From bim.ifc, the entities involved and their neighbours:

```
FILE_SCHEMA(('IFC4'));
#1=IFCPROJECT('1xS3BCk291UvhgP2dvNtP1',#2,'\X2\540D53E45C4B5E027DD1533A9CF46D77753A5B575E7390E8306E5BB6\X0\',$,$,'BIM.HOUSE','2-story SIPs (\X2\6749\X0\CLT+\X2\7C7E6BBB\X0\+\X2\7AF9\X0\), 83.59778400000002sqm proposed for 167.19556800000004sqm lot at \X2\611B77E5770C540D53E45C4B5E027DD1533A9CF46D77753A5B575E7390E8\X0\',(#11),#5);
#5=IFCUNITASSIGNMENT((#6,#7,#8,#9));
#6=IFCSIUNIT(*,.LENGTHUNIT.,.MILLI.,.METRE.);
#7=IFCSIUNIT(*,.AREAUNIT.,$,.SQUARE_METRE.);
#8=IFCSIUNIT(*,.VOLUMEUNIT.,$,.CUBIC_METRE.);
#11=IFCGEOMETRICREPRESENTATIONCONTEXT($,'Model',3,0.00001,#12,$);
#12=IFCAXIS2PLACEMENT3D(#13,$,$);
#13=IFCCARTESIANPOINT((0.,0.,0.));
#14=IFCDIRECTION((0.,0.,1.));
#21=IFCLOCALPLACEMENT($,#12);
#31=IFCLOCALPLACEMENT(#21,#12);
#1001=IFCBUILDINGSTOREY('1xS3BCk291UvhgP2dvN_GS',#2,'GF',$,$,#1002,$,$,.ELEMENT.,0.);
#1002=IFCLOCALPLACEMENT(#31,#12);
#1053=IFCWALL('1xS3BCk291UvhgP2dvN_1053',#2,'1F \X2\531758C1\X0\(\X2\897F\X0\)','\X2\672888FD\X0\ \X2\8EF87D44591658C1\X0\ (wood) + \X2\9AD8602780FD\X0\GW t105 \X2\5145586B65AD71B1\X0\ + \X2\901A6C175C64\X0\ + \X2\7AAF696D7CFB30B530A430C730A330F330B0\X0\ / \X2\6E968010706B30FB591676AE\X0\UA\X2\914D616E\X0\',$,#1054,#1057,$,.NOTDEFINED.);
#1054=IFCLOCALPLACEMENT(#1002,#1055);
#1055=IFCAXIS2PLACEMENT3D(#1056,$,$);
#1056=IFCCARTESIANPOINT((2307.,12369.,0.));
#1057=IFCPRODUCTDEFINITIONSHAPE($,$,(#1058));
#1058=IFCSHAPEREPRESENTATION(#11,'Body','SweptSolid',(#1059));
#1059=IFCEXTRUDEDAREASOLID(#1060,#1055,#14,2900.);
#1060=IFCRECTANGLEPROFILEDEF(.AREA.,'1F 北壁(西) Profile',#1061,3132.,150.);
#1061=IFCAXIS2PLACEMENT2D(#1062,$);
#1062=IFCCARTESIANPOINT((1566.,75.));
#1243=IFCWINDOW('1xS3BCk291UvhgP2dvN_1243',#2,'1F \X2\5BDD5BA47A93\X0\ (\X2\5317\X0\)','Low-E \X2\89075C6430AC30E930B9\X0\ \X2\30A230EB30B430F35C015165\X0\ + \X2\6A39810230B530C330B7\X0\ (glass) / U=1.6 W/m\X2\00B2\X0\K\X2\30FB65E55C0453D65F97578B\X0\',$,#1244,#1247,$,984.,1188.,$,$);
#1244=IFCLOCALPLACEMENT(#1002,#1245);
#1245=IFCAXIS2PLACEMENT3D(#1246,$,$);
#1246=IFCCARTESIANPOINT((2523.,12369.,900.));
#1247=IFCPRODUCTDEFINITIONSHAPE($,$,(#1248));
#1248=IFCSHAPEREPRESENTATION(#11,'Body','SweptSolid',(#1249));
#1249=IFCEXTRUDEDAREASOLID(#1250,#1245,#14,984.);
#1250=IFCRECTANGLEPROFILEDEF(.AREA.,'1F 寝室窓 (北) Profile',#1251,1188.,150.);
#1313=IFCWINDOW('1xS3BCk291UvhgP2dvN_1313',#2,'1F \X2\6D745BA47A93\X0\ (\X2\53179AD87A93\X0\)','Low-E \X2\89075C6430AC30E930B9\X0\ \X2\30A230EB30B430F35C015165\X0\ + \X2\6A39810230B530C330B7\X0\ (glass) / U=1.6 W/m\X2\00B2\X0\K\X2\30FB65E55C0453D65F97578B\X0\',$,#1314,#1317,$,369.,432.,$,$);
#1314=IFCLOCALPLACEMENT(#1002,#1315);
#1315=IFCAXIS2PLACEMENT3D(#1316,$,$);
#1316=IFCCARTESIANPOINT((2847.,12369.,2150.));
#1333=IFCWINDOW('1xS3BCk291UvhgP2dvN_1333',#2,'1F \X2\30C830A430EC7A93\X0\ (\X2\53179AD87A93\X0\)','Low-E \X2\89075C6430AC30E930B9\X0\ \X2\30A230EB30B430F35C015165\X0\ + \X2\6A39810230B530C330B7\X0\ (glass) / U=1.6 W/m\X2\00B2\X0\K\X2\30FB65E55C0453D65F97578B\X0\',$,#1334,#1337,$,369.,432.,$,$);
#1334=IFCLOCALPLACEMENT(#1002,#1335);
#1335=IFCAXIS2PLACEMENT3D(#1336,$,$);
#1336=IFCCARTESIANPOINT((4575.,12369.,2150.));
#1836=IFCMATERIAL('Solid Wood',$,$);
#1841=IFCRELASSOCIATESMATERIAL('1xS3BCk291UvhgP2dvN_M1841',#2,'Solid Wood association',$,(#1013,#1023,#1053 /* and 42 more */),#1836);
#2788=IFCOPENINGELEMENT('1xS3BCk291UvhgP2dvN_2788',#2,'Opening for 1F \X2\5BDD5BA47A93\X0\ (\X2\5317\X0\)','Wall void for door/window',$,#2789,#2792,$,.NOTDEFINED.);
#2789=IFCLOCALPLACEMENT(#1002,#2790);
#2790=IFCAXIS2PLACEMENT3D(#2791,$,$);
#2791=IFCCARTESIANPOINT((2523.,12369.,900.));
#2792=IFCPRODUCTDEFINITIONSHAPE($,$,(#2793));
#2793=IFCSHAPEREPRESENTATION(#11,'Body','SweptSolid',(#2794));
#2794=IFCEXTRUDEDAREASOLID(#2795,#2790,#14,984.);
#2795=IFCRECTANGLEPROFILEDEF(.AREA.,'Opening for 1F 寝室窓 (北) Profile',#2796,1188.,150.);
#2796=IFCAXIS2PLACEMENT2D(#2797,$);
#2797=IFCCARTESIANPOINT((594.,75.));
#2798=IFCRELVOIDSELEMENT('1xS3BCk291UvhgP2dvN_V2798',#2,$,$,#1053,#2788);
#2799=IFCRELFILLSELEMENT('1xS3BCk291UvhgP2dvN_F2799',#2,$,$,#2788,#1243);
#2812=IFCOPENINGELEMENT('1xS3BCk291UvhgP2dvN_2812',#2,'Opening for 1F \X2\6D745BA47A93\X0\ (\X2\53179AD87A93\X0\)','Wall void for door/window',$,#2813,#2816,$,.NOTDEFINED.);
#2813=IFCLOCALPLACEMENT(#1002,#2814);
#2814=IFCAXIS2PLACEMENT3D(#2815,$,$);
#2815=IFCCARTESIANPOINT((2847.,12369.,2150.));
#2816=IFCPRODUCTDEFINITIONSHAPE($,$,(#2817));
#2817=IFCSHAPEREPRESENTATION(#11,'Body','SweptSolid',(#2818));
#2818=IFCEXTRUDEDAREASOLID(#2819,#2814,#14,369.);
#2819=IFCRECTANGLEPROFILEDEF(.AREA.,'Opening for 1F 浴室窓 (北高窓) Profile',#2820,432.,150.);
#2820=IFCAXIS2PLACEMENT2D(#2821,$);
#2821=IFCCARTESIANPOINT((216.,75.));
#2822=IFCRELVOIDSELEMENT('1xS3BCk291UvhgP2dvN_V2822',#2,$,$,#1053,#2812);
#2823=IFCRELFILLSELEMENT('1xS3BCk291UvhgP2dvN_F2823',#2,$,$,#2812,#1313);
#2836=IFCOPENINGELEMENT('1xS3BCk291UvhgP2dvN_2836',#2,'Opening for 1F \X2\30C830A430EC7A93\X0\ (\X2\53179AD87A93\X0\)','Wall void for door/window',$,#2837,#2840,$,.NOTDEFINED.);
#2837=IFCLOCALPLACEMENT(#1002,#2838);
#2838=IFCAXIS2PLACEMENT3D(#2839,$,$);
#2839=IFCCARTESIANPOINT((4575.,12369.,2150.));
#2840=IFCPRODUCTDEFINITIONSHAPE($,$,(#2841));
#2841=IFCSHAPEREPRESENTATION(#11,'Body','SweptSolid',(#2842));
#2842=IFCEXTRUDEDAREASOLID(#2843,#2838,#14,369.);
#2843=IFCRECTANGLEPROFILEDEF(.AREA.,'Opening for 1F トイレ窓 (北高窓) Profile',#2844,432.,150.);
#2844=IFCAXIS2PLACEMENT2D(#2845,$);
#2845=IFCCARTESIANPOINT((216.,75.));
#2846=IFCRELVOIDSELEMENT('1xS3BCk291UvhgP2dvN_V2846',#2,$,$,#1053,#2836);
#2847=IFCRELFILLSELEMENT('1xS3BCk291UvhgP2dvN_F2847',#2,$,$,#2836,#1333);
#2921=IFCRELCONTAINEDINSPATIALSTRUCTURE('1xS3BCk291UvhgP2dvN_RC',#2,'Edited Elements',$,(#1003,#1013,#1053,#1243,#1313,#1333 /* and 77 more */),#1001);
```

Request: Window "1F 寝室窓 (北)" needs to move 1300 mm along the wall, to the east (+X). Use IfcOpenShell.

```python
import ifcopenshell
import ifcopenshell.api.geometry
import ifcopenshell.util.placement
import ifcopenshell.util.unit

model = ifcopenshell.open("bim.ifc")
unit_scale = ifcopenshell.util.unit.calculate_unit_scale(model)

window = model.by_guid("1xS3BCk291UvhgP2dvN_1243")
opening = window.FillsVoids[0].RelatingOpeningElement
wall = opening.VoidsElements[0].RelatingBuildingElement

wall_matrix = ifcopenshell.util.placement.get_local_placement(wall.ObjectPlacement)
shift = wall_matrix[:3, 0] * 1.3 / unit_scale
before = ifcopenshell.util.placement.get_local_placement(window.ObjectPlacement)[:3, 3].copy()

# The window is not placed relative to its opening, so move both.
for product in (opening, window):
    matrix = ifcopenshell.util.placement.get_local_placement(product.ObjectPlacement)
    matrix[:3, 3] += shift
    ifcopenshell.api.geometry.edit_object_placement(model, product=product, matrix=matrix, is_si=False)

after = ifcopenshell.util.placement.get_local_placement(window.ObjectPlacement)[:3, 3]
print("window moved by", (after - before).round(3) + 0.0)

model.write("bim_v2.ifc")
```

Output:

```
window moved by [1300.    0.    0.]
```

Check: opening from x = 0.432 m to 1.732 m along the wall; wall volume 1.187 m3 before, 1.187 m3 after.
